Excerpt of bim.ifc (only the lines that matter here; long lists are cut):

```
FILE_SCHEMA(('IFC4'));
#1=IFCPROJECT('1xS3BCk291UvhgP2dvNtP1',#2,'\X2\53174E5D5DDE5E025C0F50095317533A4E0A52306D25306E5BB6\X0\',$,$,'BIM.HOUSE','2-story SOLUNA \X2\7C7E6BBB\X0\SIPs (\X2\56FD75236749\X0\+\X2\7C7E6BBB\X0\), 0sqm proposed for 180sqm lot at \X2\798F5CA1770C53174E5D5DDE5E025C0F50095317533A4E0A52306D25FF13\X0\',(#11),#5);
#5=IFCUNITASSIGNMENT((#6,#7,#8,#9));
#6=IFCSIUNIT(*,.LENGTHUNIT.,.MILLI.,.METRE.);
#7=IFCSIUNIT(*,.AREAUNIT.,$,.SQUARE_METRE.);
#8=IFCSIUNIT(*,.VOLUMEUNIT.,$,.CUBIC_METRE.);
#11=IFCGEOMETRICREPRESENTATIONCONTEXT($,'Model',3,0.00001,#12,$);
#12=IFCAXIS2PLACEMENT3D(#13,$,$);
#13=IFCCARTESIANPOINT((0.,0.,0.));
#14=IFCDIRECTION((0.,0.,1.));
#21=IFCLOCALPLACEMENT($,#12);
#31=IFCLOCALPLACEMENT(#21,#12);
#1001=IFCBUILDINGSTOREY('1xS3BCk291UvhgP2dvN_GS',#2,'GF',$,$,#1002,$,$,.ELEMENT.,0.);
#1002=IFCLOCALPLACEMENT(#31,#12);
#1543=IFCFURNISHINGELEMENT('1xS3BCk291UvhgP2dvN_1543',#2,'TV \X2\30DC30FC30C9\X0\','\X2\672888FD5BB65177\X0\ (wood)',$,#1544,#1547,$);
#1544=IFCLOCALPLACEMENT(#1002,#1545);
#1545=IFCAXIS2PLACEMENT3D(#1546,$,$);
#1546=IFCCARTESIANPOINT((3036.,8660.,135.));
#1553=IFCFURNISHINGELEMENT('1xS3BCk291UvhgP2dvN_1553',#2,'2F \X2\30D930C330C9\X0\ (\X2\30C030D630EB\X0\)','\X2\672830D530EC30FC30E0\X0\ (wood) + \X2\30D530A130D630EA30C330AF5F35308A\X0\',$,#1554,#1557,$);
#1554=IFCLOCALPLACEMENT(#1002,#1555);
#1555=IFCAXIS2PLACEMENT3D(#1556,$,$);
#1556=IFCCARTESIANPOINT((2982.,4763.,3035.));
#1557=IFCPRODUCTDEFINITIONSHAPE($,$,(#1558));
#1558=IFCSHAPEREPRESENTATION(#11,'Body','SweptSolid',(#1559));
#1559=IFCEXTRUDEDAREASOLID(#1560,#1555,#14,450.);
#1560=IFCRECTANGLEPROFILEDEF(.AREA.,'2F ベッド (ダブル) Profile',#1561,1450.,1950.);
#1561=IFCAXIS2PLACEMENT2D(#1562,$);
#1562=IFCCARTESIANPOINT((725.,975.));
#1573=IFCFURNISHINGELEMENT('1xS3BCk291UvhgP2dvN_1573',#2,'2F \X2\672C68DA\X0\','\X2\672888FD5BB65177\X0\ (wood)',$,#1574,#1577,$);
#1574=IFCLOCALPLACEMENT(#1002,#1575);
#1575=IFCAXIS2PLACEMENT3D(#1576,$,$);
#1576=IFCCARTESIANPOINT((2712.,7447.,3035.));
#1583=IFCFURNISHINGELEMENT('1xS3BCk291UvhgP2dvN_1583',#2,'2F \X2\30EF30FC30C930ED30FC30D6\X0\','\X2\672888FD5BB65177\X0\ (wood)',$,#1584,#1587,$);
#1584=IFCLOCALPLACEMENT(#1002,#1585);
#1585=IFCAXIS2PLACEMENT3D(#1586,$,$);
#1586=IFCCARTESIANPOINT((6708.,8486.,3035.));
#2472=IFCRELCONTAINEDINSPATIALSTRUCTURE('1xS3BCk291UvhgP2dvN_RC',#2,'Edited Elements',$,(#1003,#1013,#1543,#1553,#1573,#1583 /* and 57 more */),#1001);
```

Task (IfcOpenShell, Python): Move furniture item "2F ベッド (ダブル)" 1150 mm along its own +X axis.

```python
import ifcopenshell
import ifcopenshell.api.geometry
import ifcopenshell.util.placement
import ifcopenshell.util.unit

model = ifcopenshell.open("bim.ifc")
unit_scale = ifcopenshell.util.unit.calculate_unit_scale(model)

item = model.by_id(1553)
matrix = ifcopenshell.util.placement.get_local_placement(item.ObjectPlacement)
matrix[:3, 3] += matrix[:3, 0] * 1.15 / unit_scale
ifcopenshell.api.geometry.edit_object_placement(model, product=item, matrix=matrix, is_si=False)

print(ifcopenshell.util.placement.get_local_placement(item.ObjectPlacement).round(3) + 0.0)

model.write("bim_rev.ifc")
```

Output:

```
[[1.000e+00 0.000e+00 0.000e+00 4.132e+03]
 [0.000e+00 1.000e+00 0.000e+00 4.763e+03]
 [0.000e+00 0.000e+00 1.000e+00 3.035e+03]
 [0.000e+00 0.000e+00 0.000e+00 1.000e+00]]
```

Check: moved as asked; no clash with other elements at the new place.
